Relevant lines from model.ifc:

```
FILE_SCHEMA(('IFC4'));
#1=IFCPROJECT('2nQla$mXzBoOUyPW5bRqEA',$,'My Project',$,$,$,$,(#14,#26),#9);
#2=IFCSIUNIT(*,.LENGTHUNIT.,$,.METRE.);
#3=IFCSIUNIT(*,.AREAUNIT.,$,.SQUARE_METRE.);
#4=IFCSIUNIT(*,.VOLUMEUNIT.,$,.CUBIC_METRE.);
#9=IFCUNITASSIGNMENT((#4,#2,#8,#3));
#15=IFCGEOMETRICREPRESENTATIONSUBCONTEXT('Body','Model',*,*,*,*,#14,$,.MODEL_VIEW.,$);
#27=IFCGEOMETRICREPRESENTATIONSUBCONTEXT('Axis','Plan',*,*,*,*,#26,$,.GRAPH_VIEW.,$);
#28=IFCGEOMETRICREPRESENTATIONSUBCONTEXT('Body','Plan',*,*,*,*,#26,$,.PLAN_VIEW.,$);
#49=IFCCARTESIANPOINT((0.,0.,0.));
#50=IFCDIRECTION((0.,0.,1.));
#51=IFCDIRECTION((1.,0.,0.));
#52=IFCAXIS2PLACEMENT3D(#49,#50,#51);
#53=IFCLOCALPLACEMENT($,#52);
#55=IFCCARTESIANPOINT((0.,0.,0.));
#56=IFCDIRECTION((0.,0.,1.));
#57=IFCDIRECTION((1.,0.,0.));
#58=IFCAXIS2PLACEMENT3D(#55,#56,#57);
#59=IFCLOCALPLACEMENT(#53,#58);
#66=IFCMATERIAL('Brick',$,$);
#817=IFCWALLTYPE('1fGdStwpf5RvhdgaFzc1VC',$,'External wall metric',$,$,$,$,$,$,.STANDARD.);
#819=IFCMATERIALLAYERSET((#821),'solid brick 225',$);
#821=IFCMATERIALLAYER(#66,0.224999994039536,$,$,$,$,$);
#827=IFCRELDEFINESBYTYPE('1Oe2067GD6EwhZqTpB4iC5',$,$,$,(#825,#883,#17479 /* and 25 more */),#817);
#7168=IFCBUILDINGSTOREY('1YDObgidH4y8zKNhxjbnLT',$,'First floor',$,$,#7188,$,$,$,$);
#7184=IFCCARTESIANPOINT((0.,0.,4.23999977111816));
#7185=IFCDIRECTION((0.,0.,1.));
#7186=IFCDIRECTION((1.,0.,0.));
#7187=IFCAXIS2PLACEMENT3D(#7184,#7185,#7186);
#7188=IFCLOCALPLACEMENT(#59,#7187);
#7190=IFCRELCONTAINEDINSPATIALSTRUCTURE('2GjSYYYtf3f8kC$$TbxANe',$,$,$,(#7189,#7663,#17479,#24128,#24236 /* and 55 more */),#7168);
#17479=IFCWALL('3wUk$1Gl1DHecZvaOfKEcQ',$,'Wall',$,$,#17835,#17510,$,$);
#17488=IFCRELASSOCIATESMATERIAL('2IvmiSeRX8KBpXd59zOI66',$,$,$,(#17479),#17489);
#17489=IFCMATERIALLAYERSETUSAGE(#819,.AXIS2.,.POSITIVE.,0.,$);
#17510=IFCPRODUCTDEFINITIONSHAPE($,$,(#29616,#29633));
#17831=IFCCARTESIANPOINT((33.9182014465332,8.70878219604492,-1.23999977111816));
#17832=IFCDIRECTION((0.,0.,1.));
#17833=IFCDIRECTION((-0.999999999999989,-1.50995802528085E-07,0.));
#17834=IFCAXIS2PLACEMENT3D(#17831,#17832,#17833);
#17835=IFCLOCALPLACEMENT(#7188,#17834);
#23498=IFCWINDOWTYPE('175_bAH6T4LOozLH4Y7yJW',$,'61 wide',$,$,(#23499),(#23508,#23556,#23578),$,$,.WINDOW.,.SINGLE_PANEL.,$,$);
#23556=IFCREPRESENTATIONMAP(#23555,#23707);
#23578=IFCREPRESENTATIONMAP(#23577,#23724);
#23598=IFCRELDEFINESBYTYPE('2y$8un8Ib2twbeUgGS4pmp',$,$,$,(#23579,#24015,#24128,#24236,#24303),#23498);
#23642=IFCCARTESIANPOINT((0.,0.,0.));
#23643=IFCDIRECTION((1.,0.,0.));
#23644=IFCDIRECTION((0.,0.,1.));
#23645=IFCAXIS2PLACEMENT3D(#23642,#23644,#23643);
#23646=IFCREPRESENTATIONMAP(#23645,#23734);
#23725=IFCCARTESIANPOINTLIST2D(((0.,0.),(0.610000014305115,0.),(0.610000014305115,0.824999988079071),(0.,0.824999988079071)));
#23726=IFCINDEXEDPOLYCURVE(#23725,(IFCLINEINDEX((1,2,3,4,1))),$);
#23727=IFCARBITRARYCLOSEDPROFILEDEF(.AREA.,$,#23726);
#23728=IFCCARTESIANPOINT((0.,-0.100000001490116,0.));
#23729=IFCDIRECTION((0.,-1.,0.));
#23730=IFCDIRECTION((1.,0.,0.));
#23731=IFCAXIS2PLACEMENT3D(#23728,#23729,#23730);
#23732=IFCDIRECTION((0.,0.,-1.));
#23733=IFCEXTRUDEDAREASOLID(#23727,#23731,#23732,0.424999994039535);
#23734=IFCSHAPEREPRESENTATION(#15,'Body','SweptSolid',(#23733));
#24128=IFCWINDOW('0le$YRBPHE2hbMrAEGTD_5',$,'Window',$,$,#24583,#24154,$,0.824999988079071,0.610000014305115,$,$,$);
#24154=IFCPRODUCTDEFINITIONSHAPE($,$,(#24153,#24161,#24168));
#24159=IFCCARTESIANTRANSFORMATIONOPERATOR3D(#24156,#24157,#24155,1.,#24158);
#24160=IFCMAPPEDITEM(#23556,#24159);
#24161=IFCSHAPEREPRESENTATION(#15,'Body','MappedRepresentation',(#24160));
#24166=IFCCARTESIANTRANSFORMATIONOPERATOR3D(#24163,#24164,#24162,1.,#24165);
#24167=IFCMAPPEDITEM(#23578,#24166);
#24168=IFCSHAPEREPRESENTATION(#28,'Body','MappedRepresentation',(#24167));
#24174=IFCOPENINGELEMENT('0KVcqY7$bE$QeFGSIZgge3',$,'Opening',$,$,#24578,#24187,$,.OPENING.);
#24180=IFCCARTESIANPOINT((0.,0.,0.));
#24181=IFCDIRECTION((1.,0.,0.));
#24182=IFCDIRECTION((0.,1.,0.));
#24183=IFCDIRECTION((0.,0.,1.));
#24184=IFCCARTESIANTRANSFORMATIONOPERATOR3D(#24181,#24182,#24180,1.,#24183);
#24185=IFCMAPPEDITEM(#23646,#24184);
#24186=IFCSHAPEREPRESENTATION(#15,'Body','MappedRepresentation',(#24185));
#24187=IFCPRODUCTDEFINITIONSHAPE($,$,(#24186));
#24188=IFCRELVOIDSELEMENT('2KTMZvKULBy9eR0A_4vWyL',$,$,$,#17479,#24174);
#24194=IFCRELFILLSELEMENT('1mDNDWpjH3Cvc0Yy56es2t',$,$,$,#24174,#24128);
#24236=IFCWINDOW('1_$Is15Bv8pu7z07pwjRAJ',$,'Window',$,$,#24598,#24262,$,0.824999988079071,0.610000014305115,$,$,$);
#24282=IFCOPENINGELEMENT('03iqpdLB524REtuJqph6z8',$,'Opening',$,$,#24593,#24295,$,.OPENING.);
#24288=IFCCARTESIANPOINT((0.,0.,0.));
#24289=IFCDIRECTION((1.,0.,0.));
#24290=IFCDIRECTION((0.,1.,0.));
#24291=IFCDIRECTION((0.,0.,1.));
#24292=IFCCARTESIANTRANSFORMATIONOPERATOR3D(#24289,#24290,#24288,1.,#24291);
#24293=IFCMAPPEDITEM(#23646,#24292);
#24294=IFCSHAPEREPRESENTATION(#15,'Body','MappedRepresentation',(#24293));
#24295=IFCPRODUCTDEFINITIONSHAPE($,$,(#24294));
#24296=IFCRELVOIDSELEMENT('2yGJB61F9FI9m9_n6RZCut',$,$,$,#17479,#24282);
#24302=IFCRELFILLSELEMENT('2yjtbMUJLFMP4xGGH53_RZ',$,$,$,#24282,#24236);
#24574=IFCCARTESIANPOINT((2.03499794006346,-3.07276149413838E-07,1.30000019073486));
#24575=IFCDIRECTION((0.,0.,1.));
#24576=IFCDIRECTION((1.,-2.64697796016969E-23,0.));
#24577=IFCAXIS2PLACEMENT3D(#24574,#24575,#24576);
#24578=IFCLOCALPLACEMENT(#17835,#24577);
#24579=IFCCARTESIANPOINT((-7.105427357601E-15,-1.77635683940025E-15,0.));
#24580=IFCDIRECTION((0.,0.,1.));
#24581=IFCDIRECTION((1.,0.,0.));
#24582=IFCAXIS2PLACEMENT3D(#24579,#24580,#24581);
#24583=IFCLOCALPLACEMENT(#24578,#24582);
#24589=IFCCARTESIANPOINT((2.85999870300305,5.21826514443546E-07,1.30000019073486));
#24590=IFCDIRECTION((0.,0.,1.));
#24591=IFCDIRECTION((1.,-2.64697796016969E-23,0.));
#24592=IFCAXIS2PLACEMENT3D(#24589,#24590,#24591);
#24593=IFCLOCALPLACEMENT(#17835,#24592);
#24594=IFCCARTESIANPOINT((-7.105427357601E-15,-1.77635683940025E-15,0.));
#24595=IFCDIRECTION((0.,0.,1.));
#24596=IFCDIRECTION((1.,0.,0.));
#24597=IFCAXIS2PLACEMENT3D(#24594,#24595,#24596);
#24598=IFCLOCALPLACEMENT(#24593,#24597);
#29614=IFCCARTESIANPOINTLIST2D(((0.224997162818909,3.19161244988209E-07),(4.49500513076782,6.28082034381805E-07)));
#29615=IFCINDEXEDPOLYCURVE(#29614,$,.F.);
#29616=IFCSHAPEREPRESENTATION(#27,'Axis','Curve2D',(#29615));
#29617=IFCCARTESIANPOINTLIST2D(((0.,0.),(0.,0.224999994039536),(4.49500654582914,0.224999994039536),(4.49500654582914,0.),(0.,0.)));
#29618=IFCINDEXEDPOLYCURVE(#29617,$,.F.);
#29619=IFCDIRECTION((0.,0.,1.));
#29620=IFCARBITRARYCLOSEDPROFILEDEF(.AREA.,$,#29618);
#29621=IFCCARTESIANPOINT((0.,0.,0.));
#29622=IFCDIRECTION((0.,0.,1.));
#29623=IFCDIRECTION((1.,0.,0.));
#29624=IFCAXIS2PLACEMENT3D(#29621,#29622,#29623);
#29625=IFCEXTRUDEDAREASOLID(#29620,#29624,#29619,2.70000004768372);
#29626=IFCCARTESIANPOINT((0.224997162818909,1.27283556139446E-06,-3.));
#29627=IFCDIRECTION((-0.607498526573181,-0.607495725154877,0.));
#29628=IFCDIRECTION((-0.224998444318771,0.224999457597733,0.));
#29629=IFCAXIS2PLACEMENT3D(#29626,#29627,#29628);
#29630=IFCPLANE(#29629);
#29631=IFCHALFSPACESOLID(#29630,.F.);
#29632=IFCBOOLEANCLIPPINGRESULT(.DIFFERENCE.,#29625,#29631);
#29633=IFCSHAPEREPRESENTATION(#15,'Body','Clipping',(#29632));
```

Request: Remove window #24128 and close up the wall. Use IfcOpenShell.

```python
import ifcopenshell
import ifcopenshell.api.feature
import ifcopenshell.api.root
import ifcopenshell.geom
import ifcopenshell.util.shape

model = ifcopenshell.open("model.ifc")
settings = ifcopenshell.geom.settings()


def volume(element):
    """Net volume in cubic metres, openings subtracted."""
    shape = ifcopenshell.geom.create_shape(settings, element)
    return ifcopenshell.util.shape.get_volume(shape.geometry)


window = model.by_guid("0le$YRBPHE2hbMrAEGTD_5")
opening = window.FillsVoids[0].RelatingOpeningElement
wall = opening.VoidsElements[0].RelatingBuildingElement
before = volume(wall)

ifcopenshell.api.root.remove_product(model, product=window)
ifcopenshell.api.feature.remove_feature(model, feature=opening)

after = volume(wall)

print(f"wall volume {before:.3f} -> {after:.3f} m3")

model.write("model_updated.ifc")
```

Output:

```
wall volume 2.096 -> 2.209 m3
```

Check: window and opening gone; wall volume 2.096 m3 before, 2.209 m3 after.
